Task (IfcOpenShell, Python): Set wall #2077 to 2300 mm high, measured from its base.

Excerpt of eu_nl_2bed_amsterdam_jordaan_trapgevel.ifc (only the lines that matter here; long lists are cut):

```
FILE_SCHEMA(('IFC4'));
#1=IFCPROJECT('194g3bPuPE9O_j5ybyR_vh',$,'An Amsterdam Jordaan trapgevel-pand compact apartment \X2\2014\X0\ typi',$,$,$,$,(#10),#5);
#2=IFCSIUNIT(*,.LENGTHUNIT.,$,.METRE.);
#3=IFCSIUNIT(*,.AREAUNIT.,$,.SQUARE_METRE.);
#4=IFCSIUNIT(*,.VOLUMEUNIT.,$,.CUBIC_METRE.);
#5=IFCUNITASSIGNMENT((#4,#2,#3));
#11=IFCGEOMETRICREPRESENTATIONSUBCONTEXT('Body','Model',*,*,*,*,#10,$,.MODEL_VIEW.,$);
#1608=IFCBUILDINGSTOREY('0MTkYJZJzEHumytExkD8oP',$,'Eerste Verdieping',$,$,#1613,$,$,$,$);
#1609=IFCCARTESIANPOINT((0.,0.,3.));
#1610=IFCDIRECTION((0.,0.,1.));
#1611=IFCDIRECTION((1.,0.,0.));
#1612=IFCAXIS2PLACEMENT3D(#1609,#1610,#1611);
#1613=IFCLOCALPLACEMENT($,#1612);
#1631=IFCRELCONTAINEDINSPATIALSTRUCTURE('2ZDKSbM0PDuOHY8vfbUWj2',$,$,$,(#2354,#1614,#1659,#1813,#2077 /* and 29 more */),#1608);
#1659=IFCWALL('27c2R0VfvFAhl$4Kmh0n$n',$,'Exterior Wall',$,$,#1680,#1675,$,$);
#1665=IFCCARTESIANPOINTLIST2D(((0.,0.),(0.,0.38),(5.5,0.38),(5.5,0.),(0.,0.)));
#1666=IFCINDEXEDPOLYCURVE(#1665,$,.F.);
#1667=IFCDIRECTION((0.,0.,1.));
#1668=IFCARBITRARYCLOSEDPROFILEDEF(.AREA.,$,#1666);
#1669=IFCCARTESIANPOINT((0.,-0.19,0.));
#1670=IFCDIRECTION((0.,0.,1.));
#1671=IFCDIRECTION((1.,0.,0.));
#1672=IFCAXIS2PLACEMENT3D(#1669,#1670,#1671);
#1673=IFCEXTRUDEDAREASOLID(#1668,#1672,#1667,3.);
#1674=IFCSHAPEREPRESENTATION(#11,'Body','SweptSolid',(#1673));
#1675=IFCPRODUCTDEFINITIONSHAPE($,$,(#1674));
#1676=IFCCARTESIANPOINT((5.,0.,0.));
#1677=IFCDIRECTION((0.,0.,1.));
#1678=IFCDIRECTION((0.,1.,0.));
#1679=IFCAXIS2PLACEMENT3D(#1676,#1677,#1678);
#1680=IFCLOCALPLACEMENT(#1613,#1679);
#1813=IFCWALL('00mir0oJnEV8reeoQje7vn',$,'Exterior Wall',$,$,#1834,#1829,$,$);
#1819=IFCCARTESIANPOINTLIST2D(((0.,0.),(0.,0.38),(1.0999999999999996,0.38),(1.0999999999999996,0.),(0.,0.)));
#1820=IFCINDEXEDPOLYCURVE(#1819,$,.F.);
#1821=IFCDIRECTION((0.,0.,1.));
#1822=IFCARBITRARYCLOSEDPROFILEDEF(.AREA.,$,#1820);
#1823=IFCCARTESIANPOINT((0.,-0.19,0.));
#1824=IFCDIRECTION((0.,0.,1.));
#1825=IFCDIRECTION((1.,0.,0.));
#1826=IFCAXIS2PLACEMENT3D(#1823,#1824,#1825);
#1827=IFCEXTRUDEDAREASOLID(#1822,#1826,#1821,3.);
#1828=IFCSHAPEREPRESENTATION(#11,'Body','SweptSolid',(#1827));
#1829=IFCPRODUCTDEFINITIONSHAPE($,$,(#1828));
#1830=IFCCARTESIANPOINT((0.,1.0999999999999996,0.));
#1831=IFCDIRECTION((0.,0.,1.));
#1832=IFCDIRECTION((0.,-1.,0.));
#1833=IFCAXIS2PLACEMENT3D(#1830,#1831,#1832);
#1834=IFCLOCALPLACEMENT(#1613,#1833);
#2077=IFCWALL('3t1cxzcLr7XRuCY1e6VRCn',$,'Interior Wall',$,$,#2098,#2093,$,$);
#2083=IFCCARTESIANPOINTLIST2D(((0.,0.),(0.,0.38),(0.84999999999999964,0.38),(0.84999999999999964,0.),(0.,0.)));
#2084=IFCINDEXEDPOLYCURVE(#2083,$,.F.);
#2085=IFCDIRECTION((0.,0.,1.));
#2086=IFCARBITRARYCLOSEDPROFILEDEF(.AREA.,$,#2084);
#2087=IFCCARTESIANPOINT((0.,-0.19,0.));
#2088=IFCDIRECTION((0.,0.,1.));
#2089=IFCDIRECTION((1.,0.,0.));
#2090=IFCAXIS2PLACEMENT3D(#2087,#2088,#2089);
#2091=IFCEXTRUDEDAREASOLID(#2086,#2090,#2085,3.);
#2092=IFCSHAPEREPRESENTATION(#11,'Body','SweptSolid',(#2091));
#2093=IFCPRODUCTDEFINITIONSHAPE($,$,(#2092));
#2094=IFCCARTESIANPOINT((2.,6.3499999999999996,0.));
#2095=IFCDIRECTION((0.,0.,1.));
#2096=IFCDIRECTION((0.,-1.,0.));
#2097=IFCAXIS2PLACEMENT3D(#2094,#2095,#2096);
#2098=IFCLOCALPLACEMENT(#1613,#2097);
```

```python
import ifcopenshell
import ifcopenshell.geom
import ifcopenshell.util.representation
import ifcopenshell.util.shape
import ifcopenshell.util.unit

model = ifcopenshell.open("eu_nl_2bed_amsterdam_jordaan_trapgevel.ifc")
unit_scale = ifcopenshell.util.unit.calculate_unit_scale(model)
settings = ifcopenshell.geom.settings()


def volume(element):
    """Net volume in cubic metres, openings subtracted."""
    shape = ifcopenshell.geom.create_shape(settings, element)
    return ifcopenshell.util.shape.get_volume(shape.geometry)


wall = model.by_guid("3t1cxzcLr7XRuCY1e6VRCn")
before = volume(wall)

body = ifcopenshell.util.representation.get_representation(wall, "Model", "Body")
solid = body.Items[0]
old_height = solid.Depth
solid.Depth = 2.3 / unit_scale
after = volume(wall)

print(f"height {old_height:g} -> {solid.Depth:g}, volume {before:.3f} -> {after:.3f} m3")

model.write("eu_nl_2bed_amsterdam_jordaan_trapgevel_rev.ifc")
```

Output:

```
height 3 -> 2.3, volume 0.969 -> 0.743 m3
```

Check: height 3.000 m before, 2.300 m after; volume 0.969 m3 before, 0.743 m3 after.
